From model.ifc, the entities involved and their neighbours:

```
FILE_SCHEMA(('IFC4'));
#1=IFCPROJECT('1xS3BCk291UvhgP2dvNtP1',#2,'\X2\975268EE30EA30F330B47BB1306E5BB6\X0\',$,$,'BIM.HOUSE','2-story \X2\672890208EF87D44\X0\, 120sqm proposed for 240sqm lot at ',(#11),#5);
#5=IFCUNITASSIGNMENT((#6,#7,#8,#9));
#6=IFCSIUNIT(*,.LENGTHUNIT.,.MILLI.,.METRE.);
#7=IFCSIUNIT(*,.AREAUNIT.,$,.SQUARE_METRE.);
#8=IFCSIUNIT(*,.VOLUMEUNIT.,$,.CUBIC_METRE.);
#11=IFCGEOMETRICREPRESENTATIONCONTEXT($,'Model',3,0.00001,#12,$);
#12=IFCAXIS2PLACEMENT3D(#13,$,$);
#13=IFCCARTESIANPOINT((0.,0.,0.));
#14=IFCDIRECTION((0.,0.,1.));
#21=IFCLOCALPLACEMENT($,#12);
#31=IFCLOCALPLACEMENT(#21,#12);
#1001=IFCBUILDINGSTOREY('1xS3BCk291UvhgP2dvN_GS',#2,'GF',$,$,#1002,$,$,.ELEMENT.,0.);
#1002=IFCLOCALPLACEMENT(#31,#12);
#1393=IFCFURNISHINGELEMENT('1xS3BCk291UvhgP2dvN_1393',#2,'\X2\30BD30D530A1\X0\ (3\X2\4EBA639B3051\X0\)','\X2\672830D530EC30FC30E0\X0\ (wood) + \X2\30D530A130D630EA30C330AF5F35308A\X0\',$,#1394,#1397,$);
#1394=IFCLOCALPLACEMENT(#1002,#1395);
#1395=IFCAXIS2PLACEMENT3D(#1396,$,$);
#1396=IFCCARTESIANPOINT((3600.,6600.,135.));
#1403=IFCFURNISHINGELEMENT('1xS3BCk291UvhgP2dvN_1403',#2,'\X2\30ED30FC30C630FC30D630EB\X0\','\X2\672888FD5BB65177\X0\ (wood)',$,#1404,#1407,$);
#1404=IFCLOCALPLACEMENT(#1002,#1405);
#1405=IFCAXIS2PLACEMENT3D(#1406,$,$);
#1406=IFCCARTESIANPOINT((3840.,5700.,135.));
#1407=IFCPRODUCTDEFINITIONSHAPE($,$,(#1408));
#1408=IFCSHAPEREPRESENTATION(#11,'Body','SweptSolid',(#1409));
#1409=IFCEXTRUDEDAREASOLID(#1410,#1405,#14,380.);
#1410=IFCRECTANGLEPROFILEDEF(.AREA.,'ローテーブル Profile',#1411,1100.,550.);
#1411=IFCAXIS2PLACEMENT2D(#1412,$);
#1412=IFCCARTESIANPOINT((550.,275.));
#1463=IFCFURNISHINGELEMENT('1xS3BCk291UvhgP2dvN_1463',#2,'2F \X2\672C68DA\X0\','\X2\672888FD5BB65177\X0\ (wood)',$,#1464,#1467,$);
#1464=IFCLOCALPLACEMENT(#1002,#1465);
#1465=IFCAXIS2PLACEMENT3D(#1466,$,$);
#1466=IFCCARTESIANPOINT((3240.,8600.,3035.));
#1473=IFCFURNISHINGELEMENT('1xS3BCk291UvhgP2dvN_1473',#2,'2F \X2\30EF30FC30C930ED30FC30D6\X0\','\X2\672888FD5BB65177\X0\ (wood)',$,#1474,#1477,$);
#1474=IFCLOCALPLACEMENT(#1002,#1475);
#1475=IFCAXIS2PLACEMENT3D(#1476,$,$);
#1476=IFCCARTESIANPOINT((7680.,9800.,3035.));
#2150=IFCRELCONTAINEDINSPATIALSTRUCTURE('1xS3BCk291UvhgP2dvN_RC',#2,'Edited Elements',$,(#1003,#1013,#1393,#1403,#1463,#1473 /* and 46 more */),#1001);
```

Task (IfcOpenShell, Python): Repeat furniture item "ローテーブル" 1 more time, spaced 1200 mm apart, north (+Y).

```python
import numpy as np
import ifcopenshell
import ifcopenshell.api.geometry
import ifcopenshell.api.root
import ifcopenshell.util.element
import ifcopenshell.util.placement

model = ifcopenshell.open("model.ifc")


def reuse_history(source, copy):
    """copy_class also copies each property set's owner history, people and application; keep the originals."""
    for rel in copy.IsDefinedBy:
        if rel.is_a("IfcRelDefinesByProperties") and (history := rel.RelatingPropertyDefinition.OwnerHistory):
            rel.RelatingPropertyDefinition.OwnerHistory = source.OwnerHistory
            ifcopenshell.util.element.remove_deep2(model, history)


source = model.by_guid("1xS3BCk291UvhgP2dvN_1403")
base = ifcopenshell.util.placement.get_local_placement(source.ObjectPlacement)
step = np.array([0.0, 1.0, 0.0]) * 1200.0

for i in range(1, 2):
    copy = ifcopenshell.api.root.copy_class(model, product=source)
    copy.Representation = ifcopenshell.util.element.copy_deep(
        model, source.Representation, exclude=["IfcGeometricRepresentationContext", "IfcRepresentationMap"]
    )
    reuse_history(source, copy)
    matrix = base.copy()
    matrix[:3, 3] += i * step
    print("added at", matrix[:3, 3].round(3) + 0.0)
    ifcopenshell.api.geometry.edit_object_placement(model, product=copy, matrix=matrix, is_si=False)

model.write("model_v2.ifc")
```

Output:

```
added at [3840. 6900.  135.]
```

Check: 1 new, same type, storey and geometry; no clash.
